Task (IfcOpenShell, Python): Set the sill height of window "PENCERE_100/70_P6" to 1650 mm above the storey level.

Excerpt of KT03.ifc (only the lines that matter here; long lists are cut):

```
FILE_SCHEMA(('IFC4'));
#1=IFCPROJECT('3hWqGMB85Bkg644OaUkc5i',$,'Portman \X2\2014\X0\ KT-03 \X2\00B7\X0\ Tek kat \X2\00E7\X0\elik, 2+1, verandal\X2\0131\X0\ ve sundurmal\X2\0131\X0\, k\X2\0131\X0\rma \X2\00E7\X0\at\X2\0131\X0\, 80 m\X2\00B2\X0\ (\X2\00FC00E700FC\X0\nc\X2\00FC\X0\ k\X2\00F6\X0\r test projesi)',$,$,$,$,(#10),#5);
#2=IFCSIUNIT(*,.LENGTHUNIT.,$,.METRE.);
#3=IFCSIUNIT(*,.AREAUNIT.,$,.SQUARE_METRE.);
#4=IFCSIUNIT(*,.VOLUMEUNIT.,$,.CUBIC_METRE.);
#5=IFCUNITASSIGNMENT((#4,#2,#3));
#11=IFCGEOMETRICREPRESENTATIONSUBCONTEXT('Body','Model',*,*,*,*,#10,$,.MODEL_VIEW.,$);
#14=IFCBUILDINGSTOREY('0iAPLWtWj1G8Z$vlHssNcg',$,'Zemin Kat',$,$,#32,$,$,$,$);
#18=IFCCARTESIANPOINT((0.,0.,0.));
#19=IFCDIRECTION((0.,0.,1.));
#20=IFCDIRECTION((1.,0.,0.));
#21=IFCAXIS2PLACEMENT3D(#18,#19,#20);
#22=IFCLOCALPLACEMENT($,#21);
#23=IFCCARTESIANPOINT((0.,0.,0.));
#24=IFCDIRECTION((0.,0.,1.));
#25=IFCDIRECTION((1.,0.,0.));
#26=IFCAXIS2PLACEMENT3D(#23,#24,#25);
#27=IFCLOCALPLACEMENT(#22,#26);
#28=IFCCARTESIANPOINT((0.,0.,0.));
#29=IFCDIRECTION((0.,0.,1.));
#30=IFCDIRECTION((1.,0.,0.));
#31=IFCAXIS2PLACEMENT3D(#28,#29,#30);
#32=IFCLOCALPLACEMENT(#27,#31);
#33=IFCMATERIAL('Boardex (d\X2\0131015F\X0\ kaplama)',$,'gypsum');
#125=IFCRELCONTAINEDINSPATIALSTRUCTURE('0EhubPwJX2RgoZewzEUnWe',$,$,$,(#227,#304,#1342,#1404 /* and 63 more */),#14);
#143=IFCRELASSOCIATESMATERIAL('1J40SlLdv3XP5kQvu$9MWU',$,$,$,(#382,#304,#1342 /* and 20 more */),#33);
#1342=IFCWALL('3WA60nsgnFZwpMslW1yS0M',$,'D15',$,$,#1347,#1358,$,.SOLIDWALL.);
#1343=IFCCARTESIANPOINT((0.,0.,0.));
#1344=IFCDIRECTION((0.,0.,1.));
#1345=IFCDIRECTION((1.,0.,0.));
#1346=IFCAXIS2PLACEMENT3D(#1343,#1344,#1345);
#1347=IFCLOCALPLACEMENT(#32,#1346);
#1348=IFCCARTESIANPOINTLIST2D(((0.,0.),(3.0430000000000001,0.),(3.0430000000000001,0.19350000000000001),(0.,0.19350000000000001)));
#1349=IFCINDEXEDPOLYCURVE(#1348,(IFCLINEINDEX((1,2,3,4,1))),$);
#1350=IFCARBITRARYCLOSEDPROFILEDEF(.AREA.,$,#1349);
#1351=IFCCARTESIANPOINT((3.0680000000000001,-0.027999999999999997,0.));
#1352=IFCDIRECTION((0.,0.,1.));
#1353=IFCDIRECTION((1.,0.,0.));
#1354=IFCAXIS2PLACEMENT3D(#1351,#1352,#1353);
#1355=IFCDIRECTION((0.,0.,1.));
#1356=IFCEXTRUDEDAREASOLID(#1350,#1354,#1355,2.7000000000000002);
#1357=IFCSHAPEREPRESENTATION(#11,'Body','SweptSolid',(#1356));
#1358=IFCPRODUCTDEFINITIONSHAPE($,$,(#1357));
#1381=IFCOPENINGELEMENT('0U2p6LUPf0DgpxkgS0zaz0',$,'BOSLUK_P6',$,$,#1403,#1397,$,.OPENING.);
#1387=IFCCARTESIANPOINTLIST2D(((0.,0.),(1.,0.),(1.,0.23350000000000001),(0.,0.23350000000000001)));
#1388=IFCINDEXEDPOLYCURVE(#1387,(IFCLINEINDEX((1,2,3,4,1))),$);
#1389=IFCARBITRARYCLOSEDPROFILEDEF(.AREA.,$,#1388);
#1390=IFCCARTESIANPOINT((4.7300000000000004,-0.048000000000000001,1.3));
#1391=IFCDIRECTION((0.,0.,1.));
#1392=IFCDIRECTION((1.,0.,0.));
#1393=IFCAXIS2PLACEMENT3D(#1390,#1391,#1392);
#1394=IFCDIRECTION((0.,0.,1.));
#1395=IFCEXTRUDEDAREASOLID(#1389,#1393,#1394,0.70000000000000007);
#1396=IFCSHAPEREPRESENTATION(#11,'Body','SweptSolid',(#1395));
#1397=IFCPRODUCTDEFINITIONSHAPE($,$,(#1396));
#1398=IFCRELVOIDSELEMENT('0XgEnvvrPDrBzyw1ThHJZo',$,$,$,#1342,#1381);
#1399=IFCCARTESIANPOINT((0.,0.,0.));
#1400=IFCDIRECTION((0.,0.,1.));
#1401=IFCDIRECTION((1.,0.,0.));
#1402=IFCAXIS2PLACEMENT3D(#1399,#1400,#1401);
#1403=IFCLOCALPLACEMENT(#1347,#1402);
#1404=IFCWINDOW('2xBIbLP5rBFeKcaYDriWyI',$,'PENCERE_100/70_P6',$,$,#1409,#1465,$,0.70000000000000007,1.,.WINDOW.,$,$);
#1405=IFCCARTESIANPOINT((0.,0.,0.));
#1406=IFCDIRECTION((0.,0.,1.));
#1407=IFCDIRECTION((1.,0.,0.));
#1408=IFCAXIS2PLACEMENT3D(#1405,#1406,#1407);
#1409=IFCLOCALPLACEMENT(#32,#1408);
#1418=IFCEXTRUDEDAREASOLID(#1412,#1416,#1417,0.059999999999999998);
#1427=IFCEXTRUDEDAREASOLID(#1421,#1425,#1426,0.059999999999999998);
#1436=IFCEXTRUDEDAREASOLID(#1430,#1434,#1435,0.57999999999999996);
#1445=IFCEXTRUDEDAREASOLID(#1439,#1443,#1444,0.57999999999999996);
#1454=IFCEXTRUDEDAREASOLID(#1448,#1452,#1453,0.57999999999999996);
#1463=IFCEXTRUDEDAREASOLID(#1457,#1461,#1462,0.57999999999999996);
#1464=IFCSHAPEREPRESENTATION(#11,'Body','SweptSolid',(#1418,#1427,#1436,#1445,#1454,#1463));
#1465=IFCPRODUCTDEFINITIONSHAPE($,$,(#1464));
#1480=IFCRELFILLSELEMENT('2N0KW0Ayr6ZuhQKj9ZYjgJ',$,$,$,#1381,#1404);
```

```python
import numpy as np
import ifcopenshell
import ifcopenshell.api.geometry
import ifcopenshell.geom
import ifcopenshell.util.element
import ifcopenshell.util.placement
import ifcopenshell.util.shape
import ifcopenshell.util.unit

model = ifcopenshell.open("KT03.ifc")
unit_scale = ifcopenshell.util.unit.calculate_unit_scale(model)

window = model.by_guid("2xBIbLP5rBFeKcaYDriWyI")
opening = window.FillsVoids[0].RelatingOpeningElement
storey = ifcopenshell.util.element.get_container(window, ifc_class="IfcBuildingStorey")
level = ifcopenshell.util.placement.get_local_placement(storey.ObjectPlacement)[2, 3]

# The opening's origin need not be at the sill, so measure its lowest point.
shape = ifcopenshell.geom.create_shape(ifcopenshell.geom.settings(), opening)
bottom = ifcopenshell.util.shape.get_shape_bottom_elevation(shape, shape.geometry) / unit_scale
dz = level + 1.65 - bottom

shift = np.array([0.0, 0.0, dz])
# The window is not placed relative to its opening, so move both.
for product in (opening, window):
    matrix = ifcopenshell.util.placement.get_local_placement(product.ObjectPlacement)
    matrix[:3, 3] += shift
    ifcopenshell.api.geometry.edit_object_placement(model, product=product, matrix=matrix, is_si=False)

print(f"moved by {dz * unit_scale:+.3f} m")

model.write("KT03_edited.ifc")
```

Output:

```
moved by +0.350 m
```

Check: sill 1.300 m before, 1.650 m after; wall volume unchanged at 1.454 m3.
